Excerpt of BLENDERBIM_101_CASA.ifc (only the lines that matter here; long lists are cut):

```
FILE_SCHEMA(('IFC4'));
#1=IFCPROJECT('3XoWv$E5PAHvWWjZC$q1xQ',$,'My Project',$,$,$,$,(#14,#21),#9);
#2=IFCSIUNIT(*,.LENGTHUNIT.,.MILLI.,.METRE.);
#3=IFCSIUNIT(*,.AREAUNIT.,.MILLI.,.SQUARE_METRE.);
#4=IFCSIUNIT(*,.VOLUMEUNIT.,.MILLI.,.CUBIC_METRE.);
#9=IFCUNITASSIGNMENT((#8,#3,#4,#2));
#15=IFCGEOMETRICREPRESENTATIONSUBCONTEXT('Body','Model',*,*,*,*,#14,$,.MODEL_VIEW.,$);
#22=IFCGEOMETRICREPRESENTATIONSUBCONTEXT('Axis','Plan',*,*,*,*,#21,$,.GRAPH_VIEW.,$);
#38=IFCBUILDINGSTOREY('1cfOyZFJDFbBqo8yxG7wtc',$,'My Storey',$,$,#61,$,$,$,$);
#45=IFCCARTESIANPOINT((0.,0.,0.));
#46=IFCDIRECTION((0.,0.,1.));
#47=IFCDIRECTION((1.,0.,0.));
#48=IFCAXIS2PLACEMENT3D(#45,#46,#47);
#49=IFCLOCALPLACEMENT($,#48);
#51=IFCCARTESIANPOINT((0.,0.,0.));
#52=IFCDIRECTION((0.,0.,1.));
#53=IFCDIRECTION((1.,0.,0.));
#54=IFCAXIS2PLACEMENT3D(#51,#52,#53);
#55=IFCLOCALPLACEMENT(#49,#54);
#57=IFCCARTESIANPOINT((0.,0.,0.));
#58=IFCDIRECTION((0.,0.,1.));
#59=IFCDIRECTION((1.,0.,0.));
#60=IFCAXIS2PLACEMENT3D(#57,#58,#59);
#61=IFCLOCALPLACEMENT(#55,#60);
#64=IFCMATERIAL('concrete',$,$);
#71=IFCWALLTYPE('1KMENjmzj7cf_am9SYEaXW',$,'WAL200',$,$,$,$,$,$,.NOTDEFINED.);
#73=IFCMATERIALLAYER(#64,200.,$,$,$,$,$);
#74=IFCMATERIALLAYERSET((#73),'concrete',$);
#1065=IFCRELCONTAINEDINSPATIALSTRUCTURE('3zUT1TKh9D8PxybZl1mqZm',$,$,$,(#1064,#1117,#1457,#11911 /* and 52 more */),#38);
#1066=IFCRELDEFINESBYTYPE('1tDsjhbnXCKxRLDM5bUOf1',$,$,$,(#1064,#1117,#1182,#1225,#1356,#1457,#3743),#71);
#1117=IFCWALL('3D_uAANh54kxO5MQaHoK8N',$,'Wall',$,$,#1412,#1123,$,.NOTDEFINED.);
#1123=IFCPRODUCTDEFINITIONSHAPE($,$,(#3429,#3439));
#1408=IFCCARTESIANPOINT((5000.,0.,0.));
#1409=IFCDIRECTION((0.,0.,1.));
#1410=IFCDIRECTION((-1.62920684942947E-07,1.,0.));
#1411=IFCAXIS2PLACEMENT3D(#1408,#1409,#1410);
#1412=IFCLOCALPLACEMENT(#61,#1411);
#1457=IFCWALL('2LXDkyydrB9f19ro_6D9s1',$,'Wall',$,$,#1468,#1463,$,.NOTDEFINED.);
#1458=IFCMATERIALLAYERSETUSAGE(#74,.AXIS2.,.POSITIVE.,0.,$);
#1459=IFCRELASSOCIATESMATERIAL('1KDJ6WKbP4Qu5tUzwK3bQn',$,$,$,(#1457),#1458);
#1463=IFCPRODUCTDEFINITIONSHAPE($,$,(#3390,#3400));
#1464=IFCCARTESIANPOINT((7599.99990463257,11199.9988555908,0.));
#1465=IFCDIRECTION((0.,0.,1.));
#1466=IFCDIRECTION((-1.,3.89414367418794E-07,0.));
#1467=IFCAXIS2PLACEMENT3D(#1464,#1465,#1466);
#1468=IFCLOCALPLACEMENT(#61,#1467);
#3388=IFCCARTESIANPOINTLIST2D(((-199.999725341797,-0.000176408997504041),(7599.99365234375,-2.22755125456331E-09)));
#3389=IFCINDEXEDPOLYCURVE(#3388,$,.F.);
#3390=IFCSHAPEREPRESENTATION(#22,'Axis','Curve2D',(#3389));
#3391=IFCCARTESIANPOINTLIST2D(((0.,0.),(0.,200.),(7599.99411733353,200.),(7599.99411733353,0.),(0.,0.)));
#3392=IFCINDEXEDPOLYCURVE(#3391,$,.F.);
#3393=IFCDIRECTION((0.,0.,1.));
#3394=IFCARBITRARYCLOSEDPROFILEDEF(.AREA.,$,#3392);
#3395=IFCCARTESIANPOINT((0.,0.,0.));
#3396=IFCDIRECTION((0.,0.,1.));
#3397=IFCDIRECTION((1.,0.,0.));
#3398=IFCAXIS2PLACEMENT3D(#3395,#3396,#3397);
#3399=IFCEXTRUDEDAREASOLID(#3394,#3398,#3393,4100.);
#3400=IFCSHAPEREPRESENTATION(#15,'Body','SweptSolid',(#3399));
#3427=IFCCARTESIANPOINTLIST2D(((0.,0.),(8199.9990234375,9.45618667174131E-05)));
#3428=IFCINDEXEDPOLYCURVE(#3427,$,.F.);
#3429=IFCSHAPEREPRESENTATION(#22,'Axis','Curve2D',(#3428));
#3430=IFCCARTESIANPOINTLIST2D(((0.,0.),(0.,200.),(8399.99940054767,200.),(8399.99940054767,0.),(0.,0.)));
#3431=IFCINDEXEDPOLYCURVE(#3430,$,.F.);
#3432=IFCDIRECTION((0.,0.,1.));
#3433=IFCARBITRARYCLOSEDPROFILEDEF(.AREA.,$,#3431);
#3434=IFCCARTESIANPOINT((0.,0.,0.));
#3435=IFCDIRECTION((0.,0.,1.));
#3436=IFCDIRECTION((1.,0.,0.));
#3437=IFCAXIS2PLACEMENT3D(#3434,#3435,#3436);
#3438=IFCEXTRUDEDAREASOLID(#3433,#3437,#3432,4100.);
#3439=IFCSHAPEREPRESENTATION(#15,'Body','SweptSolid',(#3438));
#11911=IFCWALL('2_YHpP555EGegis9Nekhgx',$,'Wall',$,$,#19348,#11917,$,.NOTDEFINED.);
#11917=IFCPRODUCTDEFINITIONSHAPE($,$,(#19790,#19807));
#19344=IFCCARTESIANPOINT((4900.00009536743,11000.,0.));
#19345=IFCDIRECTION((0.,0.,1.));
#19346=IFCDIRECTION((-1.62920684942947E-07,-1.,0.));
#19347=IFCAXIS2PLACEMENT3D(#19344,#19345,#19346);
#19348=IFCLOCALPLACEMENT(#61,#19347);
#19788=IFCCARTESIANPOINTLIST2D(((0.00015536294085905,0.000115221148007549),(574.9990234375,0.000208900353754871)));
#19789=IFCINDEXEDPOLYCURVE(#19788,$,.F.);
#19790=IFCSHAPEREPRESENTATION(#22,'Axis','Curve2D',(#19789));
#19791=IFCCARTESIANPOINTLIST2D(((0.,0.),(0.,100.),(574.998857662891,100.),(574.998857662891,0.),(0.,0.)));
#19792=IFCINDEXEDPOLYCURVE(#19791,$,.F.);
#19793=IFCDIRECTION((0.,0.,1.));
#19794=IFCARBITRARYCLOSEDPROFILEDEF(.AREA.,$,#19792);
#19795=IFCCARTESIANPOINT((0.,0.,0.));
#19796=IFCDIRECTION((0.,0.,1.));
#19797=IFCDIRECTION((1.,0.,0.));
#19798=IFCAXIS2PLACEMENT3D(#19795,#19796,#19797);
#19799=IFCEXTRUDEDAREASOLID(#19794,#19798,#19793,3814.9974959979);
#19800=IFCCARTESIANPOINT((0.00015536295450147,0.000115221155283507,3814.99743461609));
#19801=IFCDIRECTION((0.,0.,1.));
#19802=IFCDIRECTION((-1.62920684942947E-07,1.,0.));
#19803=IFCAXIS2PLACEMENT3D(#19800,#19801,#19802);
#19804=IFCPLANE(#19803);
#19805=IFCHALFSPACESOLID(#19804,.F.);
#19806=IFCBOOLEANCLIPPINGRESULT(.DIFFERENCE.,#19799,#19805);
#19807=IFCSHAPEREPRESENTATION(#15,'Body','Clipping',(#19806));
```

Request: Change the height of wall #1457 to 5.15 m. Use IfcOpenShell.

```python
import ifcopenshell
import ifcopenshell.geom
import ifcopenshell.util.representation
import ifcopenshell.util.shape
import ifcopenshell.util.unit

model = ifcopenshell.open("BLENDERBIM_101_CASA.ifc")
unit_scale = ifcopenshell.util.unit.calculate_unit_scale(model)
settings = ifcopenshell.geom.settings()


def volume(element):
    """Net volume in cubic metres, openings subtracted."""
    shape = ifcopenshell.geom.create_shape(settings, element)
    return ifcopenshell.util.shape.get_volume(shape.geometry)


wall = model.by_guid("2LXDkyydrB9f19ro_6D9s1")
before = volume(wall)

body = ifcopenshell.util.representation.get_representation(wall, "Model", "Body")
solid = body.Items[0]
old_height = solid.Depth
solid.Depth = 5.15 / unit_scale
after = volume(wall)

print(f"height {old_height:g} -> {solid.Depth:g}, volume {before:.3f} -> {after:.3f} m3")

model.write("BLENDERBIM_101_CASA_v2.ifc")
```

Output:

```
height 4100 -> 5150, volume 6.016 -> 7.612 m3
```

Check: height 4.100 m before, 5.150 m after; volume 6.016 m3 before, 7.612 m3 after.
